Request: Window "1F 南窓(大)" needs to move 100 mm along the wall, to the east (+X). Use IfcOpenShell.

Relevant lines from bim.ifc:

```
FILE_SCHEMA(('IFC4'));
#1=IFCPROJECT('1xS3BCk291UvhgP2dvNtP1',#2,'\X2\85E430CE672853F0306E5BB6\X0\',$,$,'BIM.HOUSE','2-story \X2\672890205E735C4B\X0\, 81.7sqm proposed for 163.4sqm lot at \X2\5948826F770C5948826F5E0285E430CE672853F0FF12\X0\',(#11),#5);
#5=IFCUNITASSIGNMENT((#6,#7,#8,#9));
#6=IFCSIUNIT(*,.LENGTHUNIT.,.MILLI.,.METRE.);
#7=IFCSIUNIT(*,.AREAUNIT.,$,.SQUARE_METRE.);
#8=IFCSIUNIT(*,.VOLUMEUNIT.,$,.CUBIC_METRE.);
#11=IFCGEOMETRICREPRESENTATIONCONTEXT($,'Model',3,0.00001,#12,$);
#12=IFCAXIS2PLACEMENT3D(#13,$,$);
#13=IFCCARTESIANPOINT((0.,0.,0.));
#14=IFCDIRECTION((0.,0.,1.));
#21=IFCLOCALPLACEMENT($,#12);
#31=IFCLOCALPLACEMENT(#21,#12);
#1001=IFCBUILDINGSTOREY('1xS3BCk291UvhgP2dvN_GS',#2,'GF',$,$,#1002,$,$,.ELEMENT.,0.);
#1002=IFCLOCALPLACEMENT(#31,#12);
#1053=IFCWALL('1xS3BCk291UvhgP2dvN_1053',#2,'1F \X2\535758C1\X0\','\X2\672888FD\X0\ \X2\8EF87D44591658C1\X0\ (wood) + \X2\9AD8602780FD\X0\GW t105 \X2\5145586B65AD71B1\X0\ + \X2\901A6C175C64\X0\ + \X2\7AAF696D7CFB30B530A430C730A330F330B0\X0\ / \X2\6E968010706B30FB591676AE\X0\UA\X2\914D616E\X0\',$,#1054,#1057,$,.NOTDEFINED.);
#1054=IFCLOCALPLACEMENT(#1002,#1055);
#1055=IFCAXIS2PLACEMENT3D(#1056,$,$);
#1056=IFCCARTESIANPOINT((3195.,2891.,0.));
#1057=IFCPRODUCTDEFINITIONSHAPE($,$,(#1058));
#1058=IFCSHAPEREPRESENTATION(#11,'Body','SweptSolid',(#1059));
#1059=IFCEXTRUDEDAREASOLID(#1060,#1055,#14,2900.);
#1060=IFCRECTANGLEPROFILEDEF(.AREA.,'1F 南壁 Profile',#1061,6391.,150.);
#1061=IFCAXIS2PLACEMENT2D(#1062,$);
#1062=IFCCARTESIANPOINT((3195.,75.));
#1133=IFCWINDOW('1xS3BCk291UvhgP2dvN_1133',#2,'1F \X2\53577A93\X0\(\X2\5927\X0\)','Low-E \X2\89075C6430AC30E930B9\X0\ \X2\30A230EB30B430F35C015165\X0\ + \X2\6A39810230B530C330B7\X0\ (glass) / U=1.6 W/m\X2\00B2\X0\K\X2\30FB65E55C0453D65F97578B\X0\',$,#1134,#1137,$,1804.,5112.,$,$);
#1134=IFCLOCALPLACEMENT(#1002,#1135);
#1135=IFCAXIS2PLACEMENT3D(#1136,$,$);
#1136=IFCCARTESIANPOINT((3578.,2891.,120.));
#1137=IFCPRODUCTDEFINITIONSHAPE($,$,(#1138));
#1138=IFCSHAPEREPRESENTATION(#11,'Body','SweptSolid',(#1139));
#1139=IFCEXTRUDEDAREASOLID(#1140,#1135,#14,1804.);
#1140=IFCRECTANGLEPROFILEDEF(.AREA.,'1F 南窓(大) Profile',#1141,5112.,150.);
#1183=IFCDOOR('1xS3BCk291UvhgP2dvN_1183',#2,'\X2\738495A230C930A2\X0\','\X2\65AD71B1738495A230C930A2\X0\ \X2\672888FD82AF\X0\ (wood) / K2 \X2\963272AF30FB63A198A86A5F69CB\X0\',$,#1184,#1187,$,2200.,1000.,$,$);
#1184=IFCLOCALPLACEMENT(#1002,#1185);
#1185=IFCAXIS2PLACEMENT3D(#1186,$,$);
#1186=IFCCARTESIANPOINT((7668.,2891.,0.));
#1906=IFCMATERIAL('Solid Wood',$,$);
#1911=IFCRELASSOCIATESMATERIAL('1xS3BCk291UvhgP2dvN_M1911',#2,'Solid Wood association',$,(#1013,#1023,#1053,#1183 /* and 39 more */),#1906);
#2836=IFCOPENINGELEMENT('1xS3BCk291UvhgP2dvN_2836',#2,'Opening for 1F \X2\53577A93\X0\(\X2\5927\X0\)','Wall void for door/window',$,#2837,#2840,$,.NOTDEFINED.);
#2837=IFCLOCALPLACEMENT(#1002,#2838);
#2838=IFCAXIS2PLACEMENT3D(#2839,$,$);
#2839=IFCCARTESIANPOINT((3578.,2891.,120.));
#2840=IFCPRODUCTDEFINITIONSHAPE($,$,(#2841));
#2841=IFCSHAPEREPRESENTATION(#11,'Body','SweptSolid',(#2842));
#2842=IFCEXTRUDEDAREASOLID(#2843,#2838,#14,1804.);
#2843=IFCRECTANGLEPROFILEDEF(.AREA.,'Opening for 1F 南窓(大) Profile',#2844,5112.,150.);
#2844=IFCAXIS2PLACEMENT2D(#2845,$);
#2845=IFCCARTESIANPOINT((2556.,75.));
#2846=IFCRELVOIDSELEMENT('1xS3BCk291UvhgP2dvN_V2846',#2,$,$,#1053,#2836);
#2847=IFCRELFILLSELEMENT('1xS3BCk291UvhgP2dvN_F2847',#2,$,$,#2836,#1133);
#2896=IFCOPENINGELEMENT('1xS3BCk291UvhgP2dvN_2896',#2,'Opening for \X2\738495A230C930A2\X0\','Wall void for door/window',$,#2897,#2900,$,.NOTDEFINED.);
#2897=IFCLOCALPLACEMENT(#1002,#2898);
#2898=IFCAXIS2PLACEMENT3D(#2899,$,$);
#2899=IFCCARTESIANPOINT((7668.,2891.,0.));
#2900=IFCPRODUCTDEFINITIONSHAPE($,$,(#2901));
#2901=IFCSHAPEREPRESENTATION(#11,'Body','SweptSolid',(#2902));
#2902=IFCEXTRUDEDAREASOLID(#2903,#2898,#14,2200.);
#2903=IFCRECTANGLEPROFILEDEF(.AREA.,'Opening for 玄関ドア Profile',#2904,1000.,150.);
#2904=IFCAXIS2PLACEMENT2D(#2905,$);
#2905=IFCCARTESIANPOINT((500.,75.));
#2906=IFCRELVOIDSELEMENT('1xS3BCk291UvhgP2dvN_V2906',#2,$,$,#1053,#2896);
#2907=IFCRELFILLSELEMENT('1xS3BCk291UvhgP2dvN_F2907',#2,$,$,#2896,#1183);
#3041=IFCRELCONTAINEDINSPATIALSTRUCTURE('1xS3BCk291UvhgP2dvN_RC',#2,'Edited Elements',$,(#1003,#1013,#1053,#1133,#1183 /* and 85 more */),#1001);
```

```python
import ifcopenshell
import ifcopenshell.api.geometry
import ifcopenshell.util.placement
import ifcopenshell.util.unit

model = ifcopenshell.open("bim.ifc")
unit_scale = ifcopenshell.util.unit.calculate_unit_scale(model)

window = model.by_guid("1xS3BCk291UvhgP2dvN_1133")
opening = window.FillsVoids[0].RelatingOpeningElement
wall = opening.VoidsElements[0].RelatingBuildingElement

wall_matrix = ifcopenshell.util.placement.get_local_placement(wall.ObjectPlacement)
shift = wall_matrix[:3, 0] * 0.1 / unit_scale
before = ifcopenshell.util.placement.get_local_placement(window.ObjectPlacement)[:3, 3].copy()

# The window is not placed relative to its opening, so move both.
for product in (opening, window):
    matrix = ifcopenshell.util.placement.get_local_placement(product.ObjectPlacement)
    matrix[:3, 3] += shift
    ifcopenshell.api.geometry.edit_object_placement(model, product=product, matrix=matrix, is_si=False)

after = ifcopenshell.util.placement.get_local_placement(window.ObjectPlacement)[:3, 3]
print("window moved by", (after - before).round(3) + 0.0)

model.write("bim_updated.ifc")
```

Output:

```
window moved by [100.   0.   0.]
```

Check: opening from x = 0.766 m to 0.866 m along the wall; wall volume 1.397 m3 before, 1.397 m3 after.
